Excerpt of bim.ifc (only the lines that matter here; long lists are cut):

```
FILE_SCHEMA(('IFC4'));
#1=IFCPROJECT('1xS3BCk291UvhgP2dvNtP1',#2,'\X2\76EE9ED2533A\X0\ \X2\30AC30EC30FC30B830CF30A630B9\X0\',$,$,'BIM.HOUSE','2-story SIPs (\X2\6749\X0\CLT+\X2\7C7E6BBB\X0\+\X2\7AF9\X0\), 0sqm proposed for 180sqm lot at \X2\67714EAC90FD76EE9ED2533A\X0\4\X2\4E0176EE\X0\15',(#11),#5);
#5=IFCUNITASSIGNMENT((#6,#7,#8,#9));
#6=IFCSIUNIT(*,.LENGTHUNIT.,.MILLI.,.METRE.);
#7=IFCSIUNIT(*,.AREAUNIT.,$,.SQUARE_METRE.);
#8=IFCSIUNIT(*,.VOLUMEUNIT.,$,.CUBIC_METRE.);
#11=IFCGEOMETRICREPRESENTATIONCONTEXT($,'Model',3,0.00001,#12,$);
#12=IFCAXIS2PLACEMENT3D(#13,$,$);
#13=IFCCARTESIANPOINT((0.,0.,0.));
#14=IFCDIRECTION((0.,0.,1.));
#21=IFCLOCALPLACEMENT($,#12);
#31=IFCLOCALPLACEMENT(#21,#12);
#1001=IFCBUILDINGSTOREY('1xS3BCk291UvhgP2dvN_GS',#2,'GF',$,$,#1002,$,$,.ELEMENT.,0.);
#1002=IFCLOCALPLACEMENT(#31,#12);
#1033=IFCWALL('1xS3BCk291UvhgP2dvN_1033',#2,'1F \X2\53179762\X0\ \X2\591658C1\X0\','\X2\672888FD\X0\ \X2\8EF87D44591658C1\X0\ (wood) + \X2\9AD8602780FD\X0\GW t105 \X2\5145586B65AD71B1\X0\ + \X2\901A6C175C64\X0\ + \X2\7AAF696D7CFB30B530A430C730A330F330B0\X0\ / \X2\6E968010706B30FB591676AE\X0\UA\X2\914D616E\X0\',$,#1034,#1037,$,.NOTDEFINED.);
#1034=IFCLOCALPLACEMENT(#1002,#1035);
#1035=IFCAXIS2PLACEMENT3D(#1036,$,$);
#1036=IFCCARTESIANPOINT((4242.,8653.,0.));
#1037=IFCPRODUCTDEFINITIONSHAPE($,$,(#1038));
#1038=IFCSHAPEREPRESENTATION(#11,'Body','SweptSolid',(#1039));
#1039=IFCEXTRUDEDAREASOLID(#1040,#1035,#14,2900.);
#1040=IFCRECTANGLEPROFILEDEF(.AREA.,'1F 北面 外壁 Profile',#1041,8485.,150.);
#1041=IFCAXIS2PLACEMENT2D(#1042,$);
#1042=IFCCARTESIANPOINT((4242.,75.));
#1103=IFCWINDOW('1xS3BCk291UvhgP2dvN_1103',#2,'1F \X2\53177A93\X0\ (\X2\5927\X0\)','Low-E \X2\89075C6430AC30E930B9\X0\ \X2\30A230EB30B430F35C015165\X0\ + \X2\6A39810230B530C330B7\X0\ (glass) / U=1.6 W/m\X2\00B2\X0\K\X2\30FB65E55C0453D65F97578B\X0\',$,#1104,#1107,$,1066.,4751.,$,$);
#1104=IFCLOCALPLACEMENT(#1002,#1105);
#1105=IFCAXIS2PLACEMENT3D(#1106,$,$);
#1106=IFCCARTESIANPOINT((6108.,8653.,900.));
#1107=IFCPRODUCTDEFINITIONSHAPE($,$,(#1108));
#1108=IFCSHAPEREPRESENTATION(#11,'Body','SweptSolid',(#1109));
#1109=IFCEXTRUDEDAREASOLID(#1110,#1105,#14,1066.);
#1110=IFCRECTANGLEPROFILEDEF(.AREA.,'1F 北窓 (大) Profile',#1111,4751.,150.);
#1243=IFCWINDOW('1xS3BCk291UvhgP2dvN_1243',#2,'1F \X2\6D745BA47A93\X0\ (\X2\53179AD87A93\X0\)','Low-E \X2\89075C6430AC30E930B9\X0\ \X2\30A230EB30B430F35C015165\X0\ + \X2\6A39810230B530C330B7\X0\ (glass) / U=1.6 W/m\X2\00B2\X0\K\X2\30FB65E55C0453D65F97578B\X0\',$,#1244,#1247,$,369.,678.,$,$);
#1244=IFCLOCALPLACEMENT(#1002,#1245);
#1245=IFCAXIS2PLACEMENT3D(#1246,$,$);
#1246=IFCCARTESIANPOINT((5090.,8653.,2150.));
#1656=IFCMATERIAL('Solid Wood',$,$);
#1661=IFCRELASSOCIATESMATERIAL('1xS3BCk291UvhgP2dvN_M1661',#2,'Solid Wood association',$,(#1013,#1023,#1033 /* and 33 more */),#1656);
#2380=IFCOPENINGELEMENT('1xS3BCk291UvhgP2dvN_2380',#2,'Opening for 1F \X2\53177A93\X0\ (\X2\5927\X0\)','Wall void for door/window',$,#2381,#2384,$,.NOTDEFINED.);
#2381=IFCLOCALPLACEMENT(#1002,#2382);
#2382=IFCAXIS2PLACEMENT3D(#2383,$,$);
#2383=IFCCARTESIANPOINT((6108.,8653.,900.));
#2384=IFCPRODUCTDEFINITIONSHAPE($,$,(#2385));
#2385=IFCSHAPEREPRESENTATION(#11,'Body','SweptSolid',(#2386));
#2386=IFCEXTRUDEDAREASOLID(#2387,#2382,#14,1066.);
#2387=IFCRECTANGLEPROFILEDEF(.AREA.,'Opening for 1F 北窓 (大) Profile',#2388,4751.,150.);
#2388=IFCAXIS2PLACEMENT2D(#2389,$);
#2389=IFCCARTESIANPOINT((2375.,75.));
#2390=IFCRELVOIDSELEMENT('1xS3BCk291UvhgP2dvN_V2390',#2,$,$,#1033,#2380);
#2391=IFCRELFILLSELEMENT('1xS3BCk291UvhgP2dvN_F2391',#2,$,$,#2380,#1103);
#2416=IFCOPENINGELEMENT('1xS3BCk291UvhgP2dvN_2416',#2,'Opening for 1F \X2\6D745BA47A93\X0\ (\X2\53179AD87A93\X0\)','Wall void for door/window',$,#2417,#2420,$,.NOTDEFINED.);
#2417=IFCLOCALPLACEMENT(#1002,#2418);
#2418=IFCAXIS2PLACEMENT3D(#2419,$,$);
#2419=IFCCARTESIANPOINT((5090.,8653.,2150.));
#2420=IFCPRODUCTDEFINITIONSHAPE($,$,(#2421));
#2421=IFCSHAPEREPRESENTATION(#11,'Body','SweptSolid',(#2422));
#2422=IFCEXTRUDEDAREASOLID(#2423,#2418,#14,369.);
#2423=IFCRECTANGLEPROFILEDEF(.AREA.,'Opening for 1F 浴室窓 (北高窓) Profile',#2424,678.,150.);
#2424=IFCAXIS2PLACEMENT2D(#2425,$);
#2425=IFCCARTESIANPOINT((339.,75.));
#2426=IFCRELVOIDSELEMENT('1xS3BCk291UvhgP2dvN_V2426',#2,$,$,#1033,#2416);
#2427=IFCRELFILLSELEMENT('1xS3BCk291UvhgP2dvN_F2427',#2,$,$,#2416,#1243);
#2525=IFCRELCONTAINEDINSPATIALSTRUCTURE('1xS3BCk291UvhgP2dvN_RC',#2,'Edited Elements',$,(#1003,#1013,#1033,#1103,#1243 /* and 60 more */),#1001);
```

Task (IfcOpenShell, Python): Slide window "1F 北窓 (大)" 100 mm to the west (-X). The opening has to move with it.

```python
import ifcopenshell
import ifcopenshell.api.geometry
import ifcopenshell.util.placement
import ifcopenshell.util.unit

model = ifcopenshell.open("bim.ifc")
unit_scale = ifcopenshell.util.unit.calculate_unit_scale(model)

window = model.by_id(1103)
opening = window.FillsVoids[0].RelatingOpeningElement
wall = opening.VoidsElements[0].RelatingBuildingElement

wall_matrix = ifcopenshell.util.placement.get_local_placement(wall.ObjectPlacement)
shift = wall_matrix[:3, 0] * -0.1 / unit_scale
before = ifcopenshell.util.placement.get_local_placement(window.ObjectPlacement)[:3, 3].copy()

# The window is not placed relative to its opening, so move both.
for product in (opening, window):
    matrix = ifcopenshell.util.placement.get_local_placement(product.ObjectPlacement)
    matrix[:3, 3] += shift
    ifcopenshell.api.geometry.edit_object_placement(model, product=product, matrix=matrix, is_si=False)

after = ifcopenshell.util.placement.get_local_placement(window.ObjectPlacement)[:3, 3]
print("window moved by", (after - before).round(3) + 0.0)

model.write("bim_rev.ifc")
```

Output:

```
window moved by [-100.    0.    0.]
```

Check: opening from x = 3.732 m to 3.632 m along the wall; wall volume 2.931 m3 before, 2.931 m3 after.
